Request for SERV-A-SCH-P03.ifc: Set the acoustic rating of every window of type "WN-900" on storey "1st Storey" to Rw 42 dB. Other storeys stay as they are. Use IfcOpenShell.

First a look at what the model holds.

```python
import ifcopenshell
import ifcopenshell.util.element

model = ifcopenshell.open("SERV-A-SCH-P03.ifc")
print(model.schema)
storey = next(s for s in model.by_type("IfcBuildingStorey") if s.Name == "1st Storey")
windows = [e for e in ifcopenshell.util.element.get_decomposition(storey) if e.is_a("IfcWindow")]
seen = {}
for e in windows:
    element_type = ifcopenshell.util.element.get_type(e)
    key = (element_type.Name if element_type != e and element_type else None, ifcopenshell.util.element.get_pset(e, "Pset_WindowCommon", "AcousticRating"))
    seen[key] = seen.get(key, 0) + 1
for (name, value), count in sorted(seen.items(), key=str):
    print(count, "x", name, "|", value)
```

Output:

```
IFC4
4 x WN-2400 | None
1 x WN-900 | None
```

```python
import ifcopenshell
import ifcopenshell.api.pset
import ifcopenshell.util.element

model = ifcopenshell.open("SERV-A-SCH-P03.ifc")

storey = next(s for s in model.by_type("IfcBuildingStorey") if s.Name == "1st Storey")
windows = [e for e in ifcopenshell.util.element.get_decomposition(storey) if e.is_a("IfcWindow")]

count = 0
for e in windows:
    element_type = ifcopenshell.util.element.get_type(e)
    if element_type in (None, e) or element_type.Name != "WN-900":
        continue
    # add_pset returns the element's existing set when there is one.
    pset = ifcopenshell.api.pset.add_pset(model, product=e, name="Pset_WindowCommon")
    ifcopenshell.api.pset.edit_pset(model, pset=pset, properties={"AcousticRating": "Rw 42 dB"})
    count += 1

print(count, "windows updated")

model.write("SERV-A-SCH-P03_v2.ifc")
```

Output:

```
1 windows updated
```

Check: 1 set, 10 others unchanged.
